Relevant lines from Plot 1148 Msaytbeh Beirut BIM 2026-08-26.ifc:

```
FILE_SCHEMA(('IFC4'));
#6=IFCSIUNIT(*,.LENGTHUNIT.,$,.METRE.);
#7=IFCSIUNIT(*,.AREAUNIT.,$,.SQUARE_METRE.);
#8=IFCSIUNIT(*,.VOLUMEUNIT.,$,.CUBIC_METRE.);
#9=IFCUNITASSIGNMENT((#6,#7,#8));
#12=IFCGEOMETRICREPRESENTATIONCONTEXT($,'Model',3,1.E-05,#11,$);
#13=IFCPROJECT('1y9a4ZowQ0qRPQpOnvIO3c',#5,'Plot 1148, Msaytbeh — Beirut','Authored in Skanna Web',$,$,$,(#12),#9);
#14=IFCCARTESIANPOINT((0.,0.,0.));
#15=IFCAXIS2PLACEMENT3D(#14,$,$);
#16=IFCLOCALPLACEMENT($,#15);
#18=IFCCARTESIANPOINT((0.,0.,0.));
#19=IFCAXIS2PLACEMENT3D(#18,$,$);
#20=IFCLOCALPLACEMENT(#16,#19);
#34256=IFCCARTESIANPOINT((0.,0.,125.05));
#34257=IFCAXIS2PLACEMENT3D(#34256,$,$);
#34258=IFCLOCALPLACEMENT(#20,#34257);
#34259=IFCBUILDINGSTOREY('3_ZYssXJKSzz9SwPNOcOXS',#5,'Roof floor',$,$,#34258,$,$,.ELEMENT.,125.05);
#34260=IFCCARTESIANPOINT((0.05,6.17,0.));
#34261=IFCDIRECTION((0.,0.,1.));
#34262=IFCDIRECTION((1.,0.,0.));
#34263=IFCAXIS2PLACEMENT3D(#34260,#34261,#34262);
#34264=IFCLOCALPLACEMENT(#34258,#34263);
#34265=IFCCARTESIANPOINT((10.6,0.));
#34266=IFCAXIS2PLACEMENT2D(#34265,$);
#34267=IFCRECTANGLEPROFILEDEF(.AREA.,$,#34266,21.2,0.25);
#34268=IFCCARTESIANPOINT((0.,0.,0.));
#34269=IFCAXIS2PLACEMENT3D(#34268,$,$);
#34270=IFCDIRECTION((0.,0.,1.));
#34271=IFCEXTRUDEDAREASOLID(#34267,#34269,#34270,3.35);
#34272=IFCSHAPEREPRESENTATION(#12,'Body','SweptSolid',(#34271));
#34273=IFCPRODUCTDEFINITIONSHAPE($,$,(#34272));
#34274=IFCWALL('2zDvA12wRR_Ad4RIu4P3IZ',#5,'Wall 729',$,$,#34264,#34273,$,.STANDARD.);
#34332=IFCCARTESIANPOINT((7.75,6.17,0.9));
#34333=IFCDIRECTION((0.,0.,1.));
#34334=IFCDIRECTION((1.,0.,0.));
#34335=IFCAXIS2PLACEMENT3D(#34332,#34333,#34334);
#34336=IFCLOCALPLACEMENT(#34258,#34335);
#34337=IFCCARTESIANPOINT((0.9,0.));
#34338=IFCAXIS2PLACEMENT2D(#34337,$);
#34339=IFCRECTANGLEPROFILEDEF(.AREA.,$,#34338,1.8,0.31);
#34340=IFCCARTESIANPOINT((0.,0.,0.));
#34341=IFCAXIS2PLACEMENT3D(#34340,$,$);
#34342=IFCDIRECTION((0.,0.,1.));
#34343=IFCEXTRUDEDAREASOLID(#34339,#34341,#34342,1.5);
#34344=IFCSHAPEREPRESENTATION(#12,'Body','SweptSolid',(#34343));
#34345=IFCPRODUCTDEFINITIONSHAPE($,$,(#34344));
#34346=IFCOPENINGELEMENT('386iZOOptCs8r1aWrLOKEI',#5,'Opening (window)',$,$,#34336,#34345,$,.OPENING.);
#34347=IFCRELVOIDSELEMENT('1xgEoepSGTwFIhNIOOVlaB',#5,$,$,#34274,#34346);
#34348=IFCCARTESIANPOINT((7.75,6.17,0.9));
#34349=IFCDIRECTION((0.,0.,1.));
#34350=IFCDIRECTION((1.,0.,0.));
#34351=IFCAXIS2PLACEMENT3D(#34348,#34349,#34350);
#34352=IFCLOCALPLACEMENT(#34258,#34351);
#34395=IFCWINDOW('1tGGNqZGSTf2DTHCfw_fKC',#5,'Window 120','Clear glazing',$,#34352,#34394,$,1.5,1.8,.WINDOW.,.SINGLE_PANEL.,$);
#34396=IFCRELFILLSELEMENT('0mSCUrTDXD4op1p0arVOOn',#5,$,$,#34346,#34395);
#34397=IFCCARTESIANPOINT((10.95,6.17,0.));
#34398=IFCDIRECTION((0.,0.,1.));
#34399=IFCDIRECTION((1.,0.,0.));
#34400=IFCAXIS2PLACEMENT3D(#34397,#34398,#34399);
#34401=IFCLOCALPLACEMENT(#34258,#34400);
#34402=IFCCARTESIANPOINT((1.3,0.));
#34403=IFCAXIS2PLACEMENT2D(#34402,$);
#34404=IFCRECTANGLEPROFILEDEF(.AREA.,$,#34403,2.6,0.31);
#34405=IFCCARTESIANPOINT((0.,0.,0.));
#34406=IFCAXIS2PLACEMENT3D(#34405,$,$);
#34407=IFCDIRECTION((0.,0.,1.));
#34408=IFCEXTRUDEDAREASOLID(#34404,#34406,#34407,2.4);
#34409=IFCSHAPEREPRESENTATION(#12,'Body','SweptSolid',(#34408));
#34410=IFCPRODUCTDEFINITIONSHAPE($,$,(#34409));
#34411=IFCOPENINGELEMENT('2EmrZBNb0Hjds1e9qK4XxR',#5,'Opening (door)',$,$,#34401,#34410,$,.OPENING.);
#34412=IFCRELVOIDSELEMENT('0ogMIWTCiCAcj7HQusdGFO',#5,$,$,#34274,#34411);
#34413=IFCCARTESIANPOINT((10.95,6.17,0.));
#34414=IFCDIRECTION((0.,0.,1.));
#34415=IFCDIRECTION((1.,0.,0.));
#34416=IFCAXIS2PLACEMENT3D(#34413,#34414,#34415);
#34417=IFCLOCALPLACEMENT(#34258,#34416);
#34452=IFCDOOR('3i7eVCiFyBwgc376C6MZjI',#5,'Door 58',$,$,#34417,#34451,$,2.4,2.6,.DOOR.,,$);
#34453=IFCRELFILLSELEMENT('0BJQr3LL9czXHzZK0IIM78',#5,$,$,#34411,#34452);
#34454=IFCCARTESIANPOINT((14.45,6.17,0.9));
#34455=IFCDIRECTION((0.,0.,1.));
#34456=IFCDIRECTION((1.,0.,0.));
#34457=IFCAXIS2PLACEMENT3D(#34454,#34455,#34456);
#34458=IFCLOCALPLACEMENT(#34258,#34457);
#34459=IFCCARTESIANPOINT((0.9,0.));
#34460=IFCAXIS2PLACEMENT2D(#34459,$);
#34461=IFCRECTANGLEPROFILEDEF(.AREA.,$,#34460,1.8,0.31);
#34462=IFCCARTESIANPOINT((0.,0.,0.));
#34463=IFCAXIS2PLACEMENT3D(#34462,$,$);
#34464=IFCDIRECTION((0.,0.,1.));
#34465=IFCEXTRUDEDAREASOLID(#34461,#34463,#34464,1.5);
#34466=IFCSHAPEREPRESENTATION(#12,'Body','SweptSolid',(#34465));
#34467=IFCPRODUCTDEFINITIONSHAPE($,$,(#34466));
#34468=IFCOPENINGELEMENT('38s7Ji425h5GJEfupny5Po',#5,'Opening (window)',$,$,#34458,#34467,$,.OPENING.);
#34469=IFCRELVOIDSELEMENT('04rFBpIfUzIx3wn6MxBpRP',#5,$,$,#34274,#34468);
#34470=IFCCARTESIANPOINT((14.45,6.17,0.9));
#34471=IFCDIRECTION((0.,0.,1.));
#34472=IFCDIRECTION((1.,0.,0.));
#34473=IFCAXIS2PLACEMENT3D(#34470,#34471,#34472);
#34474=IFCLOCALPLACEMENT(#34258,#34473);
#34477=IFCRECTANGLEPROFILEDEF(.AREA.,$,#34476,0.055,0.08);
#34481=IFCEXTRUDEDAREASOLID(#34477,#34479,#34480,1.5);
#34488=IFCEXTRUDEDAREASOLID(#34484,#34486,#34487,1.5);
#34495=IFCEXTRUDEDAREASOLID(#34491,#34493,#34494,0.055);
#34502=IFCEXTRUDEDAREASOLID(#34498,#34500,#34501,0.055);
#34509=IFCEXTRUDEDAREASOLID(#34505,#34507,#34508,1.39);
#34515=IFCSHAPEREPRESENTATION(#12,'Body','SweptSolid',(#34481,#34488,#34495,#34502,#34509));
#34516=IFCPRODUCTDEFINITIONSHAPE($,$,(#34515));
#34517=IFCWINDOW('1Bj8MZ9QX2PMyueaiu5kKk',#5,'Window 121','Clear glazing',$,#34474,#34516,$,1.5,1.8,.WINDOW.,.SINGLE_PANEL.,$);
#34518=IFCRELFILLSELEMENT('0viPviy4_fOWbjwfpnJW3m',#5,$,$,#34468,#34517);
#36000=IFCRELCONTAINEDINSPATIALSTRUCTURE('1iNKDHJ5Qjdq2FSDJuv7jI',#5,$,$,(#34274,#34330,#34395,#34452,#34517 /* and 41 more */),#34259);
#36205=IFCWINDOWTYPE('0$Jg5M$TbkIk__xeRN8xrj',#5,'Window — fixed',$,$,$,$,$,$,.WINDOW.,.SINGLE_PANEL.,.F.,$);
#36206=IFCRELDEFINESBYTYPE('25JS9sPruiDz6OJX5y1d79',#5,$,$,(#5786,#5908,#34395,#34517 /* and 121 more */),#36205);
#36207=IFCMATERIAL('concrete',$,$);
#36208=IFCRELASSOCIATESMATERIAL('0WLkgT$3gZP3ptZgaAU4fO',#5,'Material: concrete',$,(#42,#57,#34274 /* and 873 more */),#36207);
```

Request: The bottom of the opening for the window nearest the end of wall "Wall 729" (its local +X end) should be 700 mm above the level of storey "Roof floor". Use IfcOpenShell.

```python
import numpy as np
import ifcopenshell
import ifcopenshell.api.geometry
import ifcopenshell.geom
import ifcopenshell.util.element
import ifcopenshell.util.placement
import ifcopenshell.util.shape
import ifcopenshell.util.unit

model = ifcopenshell.open("Plot 1148 Msaytbeh Beirut BIM 2026-08-26.ifc")
unit_scale = ifcopenshell.util.unit.calculate_unit_scale(model)

window = model.by_guid("1Bj8MZ9QX2PMyueaiu5kKk")
opening = window.FillsVoids[0].RelatingOpeningElement
storey = ifcopenshell.util.element.get_container(window, ifc_class="IfcBuildingStorey")
level = ifcopenshell.util.placement.get_local_placement(storey.ObjectPlacement)[2, 3]

# The opening's origin need not be at the sill, so measure its lowest point.
shape = ifcopenshell.geom.create_shape(ifcopenshell.geom.settings(), opening)
bottom = ifcopenshell.util.shape.get_shape_bottom_elevation(shape, shape.geometry) / unit_scale
dz = level + 0.7 - bottom

shift = np.array([0.0, 0.0, dz])
# The window is not placed relative to its opening, so move both.
for product in (opening, window):
    matrix = ifcopenshell.util.placement.get_local_placement(product.ObjectPlacement)
    matrix[:3, 3] += shift
    ifcopenshell.api.geometry.edit_object_placement(model, product=product, matrix=matrix, is_si=False)

print(f"moved by {dz * unit_scale:+.3f} m")

model.write("Plot 1148 Msaytbeh Beirut BIM 2026-08-26_rev.ifc")
```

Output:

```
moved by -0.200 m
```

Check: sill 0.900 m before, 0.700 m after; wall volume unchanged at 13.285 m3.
